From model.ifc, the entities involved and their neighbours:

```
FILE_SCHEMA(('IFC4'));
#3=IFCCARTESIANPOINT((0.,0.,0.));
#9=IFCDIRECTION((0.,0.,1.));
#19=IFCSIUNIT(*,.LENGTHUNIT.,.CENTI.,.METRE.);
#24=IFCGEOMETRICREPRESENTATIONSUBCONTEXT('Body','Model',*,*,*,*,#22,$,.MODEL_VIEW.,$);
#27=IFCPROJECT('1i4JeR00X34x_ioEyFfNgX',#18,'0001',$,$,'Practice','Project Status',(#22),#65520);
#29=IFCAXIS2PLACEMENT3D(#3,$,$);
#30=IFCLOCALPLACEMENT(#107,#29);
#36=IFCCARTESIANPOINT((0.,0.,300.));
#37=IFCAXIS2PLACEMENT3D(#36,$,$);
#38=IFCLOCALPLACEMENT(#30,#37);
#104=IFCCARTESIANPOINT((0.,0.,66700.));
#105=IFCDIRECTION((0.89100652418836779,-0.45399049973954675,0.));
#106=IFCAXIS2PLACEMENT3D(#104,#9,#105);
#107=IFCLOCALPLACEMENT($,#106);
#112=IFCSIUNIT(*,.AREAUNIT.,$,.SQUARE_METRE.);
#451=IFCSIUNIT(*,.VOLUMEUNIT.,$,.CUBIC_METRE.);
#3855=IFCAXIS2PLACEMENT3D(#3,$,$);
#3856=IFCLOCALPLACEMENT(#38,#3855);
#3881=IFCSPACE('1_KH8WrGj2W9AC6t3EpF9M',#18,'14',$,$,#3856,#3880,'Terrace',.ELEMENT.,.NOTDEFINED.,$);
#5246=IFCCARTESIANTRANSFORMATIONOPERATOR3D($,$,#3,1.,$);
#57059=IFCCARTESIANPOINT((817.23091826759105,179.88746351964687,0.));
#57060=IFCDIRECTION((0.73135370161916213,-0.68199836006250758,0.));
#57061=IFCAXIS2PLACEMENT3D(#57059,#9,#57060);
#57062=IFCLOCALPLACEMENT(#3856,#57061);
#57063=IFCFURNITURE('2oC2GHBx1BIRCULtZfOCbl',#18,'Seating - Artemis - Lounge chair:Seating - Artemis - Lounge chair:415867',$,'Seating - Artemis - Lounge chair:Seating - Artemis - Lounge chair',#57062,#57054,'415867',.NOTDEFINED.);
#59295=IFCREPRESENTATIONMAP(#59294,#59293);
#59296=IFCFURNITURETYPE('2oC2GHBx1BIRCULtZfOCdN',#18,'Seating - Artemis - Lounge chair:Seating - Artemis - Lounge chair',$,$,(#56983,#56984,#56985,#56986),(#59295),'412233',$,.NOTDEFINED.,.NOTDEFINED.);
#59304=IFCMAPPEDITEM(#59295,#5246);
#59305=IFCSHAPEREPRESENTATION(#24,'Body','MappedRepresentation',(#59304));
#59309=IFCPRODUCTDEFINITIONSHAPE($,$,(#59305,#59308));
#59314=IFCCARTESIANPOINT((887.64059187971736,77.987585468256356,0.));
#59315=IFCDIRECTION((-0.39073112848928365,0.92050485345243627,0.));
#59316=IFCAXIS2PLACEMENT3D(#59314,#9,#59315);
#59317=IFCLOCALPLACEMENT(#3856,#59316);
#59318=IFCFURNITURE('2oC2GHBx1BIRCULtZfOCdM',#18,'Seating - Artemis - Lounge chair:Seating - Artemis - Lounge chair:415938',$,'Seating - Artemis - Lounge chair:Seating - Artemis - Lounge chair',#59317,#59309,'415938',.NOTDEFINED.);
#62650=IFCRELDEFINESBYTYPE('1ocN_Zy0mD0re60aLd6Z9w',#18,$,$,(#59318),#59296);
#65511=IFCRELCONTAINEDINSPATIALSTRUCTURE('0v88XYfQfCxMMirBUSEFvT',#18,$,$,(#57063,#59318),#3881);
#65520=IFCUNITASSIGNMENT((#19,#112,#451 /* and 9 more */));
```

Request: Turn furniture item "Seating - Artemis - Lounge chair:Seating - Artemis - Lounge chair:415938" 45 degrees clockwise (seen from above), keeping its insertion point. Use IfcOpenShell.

```python
import ifcopenshell
import ifcopenshell.api.geometry
import ifcopenshell.util.placement

model = ifcopenshell.open("model.ifc")

item = model.by_guid("2oC2GHBx1BIRCULtZfOCdM")
matrix = ifcopenshell.util.placement.get_local_placement(item.ObjectPlacement)
matrix = matrix @ ifcopenshell.util.placement.rotation(-45, "Z")
ifcopenshell.api.geometry.edit_object_placement(model, product=item, matrix=matrix, is_si=False)

print(ifcopenshell.util.placement.get_local_placement(item.ObjectPlacement).round(3) + 0.0)

model.write("model-out.ifc")
```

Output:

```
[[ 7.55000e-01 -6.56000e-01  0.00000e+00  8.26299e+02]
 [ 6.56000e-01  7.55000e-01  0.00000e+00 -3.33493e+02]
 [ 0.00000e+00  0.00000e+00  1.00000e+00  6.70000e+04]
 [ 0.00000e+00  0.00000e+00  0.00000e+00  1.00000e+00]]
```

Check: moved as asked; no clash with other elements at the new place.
